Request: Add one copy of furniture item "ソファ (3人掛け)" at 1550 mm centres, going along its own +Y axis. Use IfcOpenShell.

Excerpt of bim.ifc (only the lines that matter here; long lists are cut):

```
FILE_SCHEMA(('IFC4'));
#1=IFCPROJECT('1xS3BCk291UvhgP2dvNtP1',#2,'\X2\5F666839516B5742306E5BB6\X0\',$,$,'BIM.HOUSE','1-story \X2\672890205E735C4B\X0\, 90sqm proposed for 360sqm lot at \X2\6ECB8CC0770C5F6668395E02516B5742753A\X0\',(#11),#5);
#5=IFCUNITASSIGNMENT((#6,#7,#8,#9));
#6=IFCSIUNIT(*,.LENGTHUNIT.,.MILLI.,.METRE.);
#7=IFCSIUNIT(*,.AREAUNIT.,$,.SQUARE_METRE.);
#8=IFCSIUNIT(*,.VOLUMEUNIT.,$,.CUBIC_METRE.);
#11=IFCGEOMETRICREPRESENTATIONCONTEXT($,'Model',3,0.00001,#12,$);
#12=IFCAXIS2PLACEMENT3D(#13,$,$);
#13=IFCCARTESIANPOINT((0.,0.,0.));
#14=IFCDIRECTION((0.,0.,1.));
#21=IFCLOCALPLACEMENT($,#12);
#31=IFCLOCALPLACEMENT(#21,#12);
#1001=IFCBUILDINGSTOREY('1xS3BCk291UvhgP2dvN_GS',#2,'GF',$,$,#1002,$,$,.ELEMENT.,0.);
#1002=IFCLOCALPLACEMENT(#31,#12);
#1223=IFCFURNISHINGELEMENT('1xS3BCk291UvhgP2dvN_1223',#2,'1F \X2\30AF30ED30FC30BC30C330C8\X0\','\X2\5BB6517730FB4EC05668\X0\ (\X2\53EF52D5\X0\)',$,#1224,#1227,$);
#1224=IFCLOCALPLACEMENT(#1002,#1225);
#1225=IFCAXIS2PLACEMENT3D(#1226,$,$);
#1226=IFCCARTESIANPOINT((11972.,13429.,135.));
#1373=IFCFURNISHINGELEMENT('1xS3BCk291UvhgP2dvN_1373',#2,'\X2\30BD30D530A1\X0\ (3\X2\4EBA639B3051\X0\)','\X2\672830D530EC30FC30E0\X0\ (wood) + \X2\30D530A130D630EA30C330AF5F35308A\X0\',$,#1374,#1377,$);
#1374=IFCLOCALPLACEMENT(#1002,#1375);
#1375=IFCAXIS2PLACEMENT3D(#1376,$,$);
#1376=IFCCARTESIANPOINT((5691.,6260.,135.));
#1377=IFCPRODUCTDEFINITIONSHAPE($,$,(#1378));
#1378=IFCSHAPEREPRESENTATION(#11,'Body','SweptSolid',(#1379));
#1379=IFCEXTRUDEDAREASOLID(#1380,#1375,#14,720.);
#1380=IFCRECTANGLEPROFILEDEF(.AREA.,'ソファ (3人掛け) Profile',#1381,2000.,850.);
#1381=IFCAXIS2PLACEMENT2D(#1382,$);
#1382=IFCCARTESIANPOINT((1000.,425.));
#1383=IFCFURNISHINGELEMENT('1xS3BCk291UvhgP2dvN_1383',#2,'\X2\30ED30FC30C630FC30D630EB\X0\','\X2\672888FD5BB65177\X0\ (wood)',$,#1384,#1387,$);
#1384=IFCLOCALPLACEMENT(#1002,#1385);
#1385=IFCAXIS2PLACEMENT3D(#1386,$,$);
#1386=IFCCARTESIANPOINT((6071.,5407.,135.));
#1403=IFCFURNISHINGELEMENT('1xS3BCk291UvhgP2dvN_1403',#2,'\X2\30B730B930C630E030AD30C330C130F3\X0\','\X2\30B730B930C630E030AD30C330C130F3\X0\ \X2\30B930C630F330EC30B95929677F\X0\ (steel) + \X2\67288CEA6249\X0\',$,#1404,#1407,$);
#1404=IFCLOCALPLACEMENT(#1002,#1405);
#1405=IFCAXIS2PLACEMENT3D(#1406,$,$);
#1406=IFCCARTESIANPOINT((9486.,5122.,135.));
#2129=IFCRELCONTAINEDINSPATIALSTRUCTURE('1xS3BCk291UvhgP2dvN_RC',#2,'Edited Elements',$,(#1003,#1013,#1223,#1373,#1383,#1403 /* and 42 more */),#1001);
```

```python
import ifcopenshell
import ifcopenshell.api.geometry
import ifcopenshell.api.root
import ifcopenshell.util.element
import ifcopenshell.util.placement

model = ifcopenshell.open("bim.ifc")


def reuse_history(source, copy):
    """copy_class also copies each property set's owner history, people and application; keep the originals."""
    for rel in copy.IsDefinedBy:
        if rel.is_a("IfcRelDefinesByProperties") and (history := rel.RelatingPropertyDefinition.OwnerHistory):
            rel.RelatingPropertyDefinition.OwnerHistory = source.OwnerHistory
            ifcopenshell.util.element.remove_deep2(model, history)


source = model.by_id(1373)
base = ifcopenshell.util.placement.get_local_placement(source.ObjectPlacement)
step = base[:3, 1] * 1550.0

for i in range(1, 2):
    copy = ifcopenshell.api.root.copy_class(model, product=source)
    copy.Representation = ifcopenshell.util.element.copy_deep(
        model, source.Representation, exclude=["IfcGeometricRepresentationContext", "IfcRepresentationMap"]
    )
    reuse_history(source, copy)
    matrix = base.copy()
    matrix[:3, 3] += i * step
    print("added at", matrix[:3, 3].round(3) + 0.0)
    ifcopenshell.api.geometry.edit_object_placement(model, product=copy, matrix=matrix, is_si=False)

model.write("bim_v2.ifc")
```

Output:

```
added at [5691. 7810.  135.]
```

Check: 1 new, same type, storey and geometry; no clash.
